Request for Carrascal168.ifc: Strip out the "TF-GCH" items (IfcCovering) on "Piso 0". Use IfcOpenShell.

First a look at what the model holds.

```python
import ifcopenshell
import ifcopenshell.util.element

model = ifcopenshell.open("Carrascal168.ifc")
print(model.schema)
storey = next(s for s in model.by_type("IfcBuildingStorey") if s.Name == "Piso 0")
coverings = [e for e in ifcopenshell.util.element.get_decomposition(storey) if e.is_a("IfcCovering")]
seen = {}
for e in coverings:
    element_type = ifcopenshell.util.element.get_type(e)
    name = element_type.Name if element_type not in (None, e) else None
    seen[name] = seen.get(name, 0) + 1
for name, count in sorted(seen.items(), key=str):
    print(count, "x", name)
```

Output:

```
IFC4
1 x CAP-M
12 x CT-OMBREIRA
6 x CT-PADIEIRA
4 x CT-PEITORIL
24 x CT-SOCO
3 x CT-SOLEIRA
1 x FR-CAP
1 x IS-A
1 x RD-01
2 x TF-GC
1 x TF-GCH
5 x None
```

```python
import ifcopenshell
import ifcopenshell.api.root
import ifcopenshell.util.element

model = ifcopenshell.open("Carrascal168.ifc")

storey = next(s for s in model.by_type("IfcBuildingStorey") if s.Name == "Piso 0")
coverings = [e for e in ifcopenshell.util.element.get_decomposition(storey) if e.is_a("IfcCovering")]
targets = [e for e in coverings if (t := ifcopenshell.util.element.get_type(e)) not in (None, e) and t.Name == "TF-GCH"]

for e in targets:
    ifcopenshell.api.root.remove_product(model, product=e)
print(len(targets), "removed")

model.write("Carrascal168-out.ifc")
```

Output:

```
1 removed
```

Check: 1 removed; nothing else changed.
